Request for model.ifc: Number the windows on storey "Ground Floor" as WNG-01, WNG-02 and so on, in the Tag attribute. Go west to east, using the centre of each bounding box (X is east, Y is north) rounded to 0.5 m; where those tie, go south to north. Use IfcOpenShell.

First a look at what the model holds.

```python
import ifcopenshell
import ifcopenshell.util.element
import ifcopenshell.util.placement

model = ifcopenshell.open("model.ifc")
print(model.schema)
storey = next(s for s in model.by_type("IfcBuildingStorey") if s.Name == "Ground Floor")
windows = [e for e in ifcopenshell.util.element.get_decomposition(storey) if e.is_a("IfcWindow")]
for e in sorted(windows, key=lambda e: e.id()):
    origin = ifcopenshell.util.placement.get_local_placement(e.ObjectPlacement)[:3, 3]
    print(e.id(), e.Tag, e.Name, origin.round(2) + 0.0, sep=" | ")
```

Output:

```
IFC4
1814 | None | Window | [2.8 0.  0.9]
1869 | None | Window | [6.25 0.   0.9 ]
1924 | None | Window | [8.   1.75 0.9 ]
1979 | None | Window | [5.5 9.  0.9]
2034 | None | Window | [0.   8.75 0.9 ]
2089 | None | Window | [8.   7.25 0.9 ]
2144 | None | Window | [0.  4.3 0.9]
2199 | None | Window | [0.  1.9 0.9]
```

```python
import ifcopenshell
import ifcopenshell.geom
import ifcopenshell.util.element
import ifcopenshell.util.shape

model = ifcopenshell.open("model.ifc")
settings = ifcopenshell.geom.settings()
settings.set("use-world-coords", True)


def centre(element):
    shape = ifcopenshell.geom.create_shape(settings, element)
    return ifcopenshell.util.shape.get_bbox_centroid(shape.geometry)


storey = next(s for s in model.by_type("IfcBuildingStorey") if s.Name == "Ground Floor")
windows = [e for e in ifcopenshell.util.element.get_decomposition(storey) if e.is_a("IfcWindow")]

# Insertion points can sit at a corner or the storey origin, so sort by the geometry (in metres).
centres = {e: centre(e) for e in windows}
windows.sort(key=lambda e: (round(centres[e][0] / 0.5), centres[e][1]))

for i, e in enumerate(windows, start=1):
    number = f"WNG-{i:02d}"
    e.Tag = number
    print(e.id(), number)

model.write("model_rev.ifc")
```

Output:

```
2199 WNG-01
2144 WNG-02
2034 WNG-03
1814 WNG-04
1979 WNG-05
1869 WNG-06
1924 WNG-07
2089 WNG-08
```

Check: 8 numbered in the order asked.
